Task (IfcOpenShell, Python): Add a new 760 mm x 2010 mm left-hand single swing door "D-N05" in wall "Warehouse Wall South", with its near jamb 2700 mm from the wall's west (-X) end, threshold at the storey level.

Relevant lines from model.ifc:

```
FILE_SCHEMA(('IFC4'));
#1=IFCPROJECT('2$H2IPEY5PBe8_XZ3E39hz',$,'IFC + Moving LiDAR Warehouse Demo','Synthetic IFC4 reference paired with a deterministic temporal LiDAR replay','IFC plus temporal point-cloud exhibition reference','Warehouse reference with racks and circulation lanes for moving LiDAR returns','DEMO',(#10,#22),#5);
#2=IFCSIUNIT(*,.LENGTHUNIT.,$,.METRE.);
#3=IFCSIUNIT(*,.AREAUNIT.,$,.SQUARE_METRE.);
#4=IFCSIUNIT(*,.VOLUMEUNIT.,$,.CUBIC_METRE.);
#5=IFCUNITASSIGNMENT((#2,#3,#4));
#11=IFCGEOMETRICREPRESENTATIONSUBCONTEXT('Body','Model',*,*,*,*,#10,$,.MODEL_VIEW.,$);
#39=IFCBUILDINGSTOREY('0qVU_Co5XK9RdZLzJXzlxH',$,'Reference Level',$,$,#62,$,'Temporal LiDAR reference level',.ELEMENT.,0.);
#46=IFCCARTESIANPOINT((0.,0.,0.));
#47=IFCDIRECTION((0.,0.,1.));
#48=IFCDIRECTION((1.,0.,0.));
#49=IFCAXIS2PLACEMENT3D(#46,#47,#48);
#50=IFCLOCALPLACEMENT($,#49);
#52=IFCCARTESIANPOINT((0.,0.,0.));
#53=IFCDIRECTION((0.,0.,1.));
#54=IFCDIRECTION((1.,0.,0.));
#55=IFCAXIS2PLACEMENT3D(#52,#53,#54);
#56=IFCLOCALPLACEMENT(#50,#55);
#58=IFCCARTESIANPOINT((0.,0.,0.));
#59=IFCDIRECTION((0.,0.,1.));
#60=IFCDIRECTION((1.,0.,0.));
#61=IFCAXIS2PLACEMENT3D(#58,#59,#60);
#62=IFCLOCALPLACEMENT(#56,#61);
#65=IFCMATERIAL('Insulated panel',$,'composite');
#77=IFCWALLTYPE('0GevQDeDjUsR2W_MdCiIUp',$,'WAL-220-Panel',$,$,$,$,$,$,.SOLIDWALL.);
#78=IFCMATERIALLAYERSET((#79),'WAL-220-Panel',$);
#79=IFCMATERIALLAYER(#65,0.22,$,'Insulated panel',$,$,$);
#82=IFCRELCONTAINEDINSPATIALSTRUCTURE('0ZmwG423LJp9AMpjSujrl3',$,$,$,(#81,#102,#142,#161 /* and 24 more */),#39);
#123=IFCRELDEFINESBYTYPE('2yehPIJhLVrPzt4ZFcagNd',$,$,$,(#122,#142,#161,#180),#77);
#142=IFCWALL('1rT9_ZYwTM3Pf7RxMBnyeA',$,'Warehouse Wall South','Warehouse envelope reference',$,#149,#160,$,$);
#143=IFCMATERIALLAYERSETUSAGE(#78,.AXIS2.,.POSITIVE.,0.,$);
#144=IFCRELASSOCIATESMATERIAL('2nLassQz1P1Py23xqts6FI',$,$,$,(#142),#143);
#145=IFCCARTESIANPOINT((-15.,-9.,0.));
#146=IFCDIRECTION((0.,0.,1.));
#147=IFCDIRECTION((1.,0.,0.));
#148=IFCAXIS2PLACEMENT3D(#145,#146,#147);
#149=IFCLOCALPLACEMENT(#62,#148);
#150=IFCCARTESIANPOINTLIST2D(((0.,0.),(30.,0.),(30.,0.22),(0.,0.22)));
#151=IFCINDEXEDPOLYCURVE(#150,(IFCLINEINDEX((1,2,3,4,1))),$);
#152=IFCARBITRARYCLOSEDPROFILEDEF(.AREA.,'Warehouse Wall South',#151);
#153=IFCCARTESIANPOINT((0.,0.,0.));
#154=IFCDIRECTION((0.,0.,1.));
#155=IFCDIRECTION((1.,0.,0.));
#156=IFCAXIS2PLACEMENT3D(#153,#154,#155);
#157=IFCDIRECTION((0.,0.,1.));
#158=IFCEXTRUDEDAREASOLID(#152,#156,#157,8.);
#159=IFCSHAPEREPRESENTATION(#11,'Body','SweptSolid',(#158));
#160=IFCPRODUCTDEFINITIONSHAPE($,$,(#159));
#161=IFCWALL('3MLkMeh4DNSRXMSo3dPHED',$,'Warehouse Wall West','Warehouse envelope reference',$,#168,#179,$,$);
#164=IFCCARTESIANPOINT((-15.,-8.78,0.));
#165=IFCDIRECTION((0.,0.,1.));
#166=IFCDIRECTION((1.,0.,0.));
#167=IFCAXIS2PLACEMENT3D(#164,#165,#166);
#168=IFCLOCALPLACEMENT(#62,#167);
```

```python
import numpy as np
import ifcopenshell
import ifcopenshell.api.feature
import ifcopenshell.api.geometry
import ifcopenshell.api.root
import ifcopenshell.api.spatial
import ifcopenshell.geom
import ifcopenshell.util.element
import ifcopenshell.util.placement
import ifcopenshell.util.representation
import ifcopenshell.util.shape
import ifcopenshell.util.unit

model = ifcopenshell.open("model.ifc")
unit_scale = ifcopenshell.util.unit.calculate_unit_scale(model)
settings = ifcopenshell.geom.settings()


def volume(element):
    """Net volume in cubic metres, openings subtracted."""
    shape = ifcopenshell.geom.create_shape(settings, element)
    return ifcopenshell.util.shape.get_volume(shape.geometry)


wall = model.by_guid("1rT9_ZYwTM3Pf7RxMBnyeA")
storey = ifcopenshell.util.element.get_container(wall, ifc_class="IfcBuildingStorey")
context = ifcopenshell.util.representation.get_context(model, "Model", "Body", "MODEL_VIEW")
before = volume(wall)

width, height, from_end, sill = 0.76, 2.01, 2.7, 0.0  # metres

# The wall runs along its own X axis, and the end named is its -X end.
wall_shape = ifcopenshell.geom.create_shape(settings, wall)
x, y, z = ifcopenshell.util.shape.get_vertices(wall_shape.geometry).T
start = x.min() + from_end
face, thickness = float(y.min()), float(y.max() - y.min())
wall_matrix = ifcopenshell.util.placement.get_local_placement(wall.ObjectPlacement)
level = ifcopenshell.util.placement.get_local_placement(storey.ObjectPlacement)[2, 3]


def in_wall(x, y):
    """Placement at x, y metres in the wall's axes, at sill height."""
    matrix = wall_matrix.copy()
    matrix[:, 3] = wall_matrix @ np.array([x / unit_scale, y / unit_scale, 0.0, 1.0])
    matrix[2, 3] = level + sill / unit_scale
    return matrix


# Opening: a box that overshoots both wall faces by 50 mm.
opening = ifcopenshell.api.root.create_entity(model, ifc_class="IfcOpeningElement", predefined_type="OPENING")
box = ifcopenshell.api.geometry.add_wall_representation(
    model, context=context, length=width, height=height, thickness=thickness + 0.1
)
ifcopenshell.api.geometry.assign_representation(model, product=opening, representation=box)
ifcopenshell.api.geometry.edit_object_placement(model, product=opening, matrix=in_wall(start, face - 0.05), is_si=False)
ifcopenshell.api.feature.add_feature(model, feature=opening, element=wall)

door = ifcopenshell.api.root.create_entity(model, ifc_class="IfcDoor", name="D-N05", predefined_type="DOOR")
door.OverallWidth, door.OverallHeight = width / unit_scale, height / unit_scale
door.OperationType = "SINGLE_SWING_LEFT"
body = ifcopenshell.api.geometry.add_door_representation(
    model,
    context=context,
    overall_width=door.OverallWidth,
    overall_height=door.OverallHeight,
    operation_type="SINGLE_SWING_LEFT",
    lining_properties={"LiningDepth": thickness / unit_scale, "ThresholdDepth": thickness / unit_scale},
)
ifcopenshell.api.geometry.assign_representation(model, product=door, representation=body)
ifcopenshell.api.spatial.assign_container(model, products=[door], relating_structure=storey)
ifcopenshell.api.feature.add_filling(model, opening=opening, element=door)

# The lining spans the wall, so the door starts at the wall face.
ifcopenshell.api.geometry.edit_object_placement(model, product=door, matrix=in_wall(start, face), is_si=False)

after = volume(wall)

print(f"wall volume {before:.3f} -> {after:.3f} m3")

model.write("model_v2.ifc")
```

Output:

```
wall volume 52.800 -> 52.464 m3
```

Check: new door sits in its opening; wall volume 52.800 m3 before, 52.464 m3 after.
